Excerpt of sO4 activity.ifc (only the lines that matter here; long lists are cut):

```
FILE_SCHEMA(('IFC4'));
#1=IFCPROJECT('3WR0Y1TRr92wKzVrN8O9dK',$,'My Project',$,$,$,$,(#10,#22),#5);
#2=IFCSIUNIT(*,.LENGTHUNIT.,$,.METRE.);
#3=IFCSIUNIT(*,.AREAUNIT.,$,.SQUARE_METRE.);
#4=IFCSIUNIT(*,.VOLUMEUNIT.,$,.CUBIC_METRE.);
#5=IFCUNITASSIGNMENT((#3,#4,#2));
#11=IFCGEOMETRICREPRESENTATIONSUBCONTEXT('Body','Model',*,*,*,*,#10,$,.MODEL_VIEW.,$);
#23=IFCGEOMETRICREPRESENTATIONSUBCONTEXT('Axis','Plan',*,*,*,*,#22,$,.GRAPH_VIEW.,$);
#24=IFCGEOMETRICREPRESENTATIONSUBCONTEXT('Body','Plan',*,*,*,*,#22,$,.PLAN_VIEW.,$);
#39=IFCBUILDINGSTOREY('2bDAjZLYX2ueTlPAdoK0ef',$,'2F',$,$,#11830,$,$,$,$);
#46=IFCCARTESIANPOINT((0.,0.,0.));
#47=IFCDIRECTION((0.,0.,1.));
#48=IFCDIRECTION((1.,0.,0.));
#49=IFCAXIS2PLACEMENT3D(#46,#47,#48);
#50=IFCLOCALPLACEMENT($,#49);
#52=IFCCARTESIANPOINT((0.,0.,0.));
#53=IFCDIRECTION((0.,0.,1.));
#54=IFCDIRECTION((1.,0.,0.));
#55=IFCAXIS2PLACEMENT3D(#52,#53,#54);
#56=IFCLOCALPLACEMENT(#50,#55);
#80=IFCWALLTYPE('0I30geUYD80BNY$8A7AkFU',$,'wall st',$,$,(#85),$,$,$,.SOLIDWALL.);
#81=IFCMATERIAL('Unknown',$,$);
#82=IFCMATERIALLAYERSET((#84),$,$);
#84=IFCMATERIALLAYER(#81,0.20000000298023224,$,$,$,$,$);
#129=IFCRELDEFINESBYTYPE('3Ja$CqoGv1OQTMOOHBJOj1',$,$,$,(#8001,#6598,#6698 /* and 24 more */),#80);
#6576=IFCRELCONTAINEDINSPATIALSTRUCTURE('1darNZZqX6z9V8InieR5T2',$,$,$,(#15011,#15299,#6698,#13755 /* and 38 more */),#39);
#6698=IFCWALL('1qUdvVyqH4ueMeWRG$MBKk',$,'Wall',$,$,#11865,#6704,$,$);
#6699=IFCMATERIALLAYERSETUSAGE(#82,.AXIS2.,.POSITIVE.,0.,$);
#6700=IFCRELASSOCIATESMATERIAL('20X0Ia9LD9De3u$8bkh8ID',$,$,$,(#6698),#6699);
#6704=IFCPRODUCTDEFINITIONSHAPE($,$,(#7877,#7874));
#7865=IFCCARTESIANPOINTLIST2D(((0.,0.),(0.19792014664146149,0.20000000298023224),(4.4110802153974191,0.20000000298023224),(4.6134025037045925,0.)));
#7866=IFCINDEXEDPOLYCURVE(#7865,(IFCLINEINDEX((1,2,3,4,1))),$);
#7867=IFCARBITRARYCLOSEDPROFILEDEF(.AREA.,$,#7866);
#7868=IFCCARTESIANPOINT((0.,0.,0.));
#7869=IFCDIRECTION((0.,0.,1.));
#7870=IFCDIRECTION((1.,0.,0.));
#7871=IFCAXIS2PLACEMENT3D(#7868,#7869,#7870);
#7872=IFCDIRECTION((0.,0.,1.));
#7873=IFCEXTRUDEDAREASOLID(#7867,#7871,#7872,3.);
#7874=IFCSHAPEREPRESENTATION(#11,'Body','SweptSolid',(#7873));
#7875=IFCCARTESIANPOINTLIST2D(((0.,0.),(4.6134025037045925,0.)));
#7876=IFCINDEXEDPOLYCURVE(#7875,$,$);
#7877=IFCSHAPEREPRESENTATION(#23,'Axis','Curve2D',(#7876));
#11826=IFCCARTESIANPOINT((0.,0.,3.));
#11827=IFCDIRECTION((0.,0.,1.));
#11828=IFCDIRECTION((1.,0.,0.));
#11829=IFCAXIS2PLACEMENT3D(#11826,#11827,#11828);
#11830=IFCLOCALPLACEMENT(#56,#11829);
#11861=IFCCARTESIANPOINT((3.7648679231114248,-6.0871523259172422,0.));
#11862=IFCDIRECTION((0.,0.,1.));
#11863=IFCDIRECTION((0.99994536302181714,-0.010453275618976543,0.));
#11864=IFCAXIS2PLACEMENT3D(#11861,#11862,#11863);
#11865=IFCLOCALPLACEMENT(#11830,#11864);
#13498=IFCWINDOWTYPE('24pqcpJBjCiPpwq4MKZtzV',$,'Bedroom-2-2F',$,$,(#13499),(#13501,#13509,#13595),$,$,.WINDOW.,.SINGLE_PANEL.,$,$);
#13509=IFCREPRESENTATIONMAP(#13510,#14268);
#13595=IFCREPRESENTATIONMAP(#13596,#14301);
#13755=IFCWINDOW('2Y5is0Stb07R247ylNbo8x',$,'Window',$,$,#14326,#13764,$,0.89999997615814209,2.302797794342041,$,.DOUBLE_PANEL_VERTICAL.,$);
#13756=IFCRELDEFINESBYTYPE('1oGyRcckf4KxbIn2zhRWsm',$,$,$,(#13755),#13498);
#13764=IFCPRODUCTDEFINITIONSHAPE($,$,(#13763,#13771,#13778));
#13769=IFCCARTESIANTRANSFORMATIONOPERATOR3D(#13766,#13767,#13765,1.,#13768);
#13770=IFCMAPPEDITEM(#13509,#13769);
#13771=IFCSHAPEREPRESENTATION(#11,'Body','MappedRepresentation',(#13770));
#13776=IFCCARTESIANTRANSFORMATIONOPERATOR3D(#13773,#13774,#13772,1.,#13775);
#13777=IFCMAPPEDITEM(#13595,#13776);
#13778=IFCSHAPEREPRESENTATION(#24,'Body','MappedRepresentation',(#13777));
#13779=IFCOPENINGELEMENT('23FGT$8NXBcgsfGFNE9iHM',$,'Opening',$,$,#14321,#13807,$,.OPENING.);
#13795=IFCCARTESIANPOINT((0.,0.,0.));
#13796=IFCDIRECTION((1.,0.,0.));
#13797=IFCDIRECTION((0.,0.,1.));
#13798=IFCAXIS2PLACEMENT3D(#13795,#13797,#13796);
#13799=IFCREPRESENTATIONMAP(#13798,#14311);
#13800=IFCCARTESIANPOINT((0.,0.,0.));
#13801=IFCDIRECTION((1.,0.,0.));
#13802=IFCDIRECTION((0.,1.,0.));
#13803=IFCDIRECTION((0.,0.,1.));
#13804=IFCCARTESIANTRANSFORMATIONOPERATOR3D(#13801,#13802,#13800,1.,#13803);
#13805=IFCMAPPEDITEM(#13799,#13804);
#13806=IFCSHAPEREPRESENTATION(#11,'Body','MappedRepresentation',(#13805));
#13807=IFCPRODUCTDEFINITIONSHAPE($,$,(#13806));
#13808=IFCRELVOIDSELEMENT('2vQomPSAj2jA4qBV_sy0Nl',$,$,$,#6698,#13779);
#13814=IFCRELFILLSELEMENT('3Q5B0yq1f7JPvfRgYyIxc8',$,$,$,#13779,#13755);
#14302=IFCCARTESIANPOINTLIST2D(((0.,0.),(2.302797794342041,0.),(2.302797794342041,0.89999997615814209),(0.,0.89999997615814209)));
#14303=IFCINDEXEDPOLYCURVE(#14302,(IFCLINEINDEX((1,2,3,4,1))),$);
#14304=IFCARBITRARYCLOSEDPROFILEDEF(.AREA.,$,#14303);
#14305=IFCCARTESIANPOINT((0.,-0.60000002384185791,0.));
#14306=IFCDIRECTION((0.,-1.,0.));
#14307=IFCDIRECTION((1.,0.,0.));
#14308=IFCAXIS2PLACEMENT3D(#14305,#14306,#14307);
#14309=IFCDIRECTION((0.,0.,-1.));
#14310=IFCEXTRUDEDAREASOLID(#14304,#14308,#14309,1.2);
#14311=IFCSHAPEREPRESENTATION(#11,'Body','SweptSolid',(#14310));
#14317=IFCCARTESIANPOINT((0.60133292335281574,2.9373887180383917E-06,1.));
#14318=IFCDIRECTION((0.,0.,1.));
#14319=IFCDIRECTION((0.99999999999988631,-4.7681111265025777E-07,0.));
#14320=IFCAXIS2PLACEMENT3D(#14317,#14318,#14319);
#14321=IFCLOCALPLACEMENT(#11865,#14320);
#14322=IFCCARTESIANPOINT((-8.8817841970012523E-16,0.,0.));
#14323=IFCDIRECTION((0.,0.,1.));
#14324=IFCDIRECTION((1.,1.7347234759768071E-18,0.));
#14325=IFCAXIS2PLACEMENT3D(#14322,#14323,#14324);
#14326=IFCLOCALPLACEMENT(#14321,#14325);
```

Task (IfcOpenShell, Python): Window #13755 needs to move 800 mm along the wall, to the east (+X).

```python
import ifcopenshell
import ifcopenshell.api.geometry
import ifcopenshell.util.placement

model = ifcopenshell.open("sO4 activity.ifc")

window = model.by_guid("2Y5is0Stb07R247ylNbo8x")
opening = window.FillsVoids[0].RelatingOpeningElement
wall = opening.VoidsElements[0].RelatingBuildingElement

wall_matrix = ifcopenshell.util.placement.get_local_placement(wall.ObjectPlacement)
shift = wall_matrix[:3, 0] * 0.8
before = ifcopenshell.util.placement.get_local_placement(window.ObjectPlacement)[:3, 3].copy()

# The window is placed relative to its opening, so it follows when the opening moves.
matrix = ifcopenshell.util.placement.get_local_placement(opening.ObjectPlacement)
matrix[:3, 3] += shift
ifcopenshell.api.geometry.edit_object_placement(
    model, product=opening, matrix=matrix, is_si=False, should_transform_children=True
)

after = ifcopenshell.util.placement.get_local_placement(window.ObjectPlacement)[:3, 3]
print("window moved by", (after - before).round(3) + 0.0)

model.write("sO4 activity_rev.ifc")
```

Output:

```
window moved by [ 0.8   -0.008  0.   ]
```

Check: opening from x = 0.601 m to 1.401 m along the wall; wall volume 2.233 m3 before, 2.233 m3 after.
